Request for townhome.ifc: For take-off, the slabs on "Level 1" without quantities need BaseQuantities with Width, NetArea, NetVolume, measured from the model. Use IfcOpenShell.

First a look at what the model holds.

```python
import ifcopenshell
import ifcopenshell.util.element
import ifcopenshell.util.unit

model = ifcopenshell.open("townhome.ifc")
print(model.schema)
for unit_type in ("LENGTHUNIT", "AREAUNIT", "VOLUMEUNIT"):
    print(unit_type, ifcopenshell.util.unit.calculate_unit_scale(model, unit_type))
storey = next(s for s in model.by_type("IfcBuildingStorey") if s.Name == "Level 1")
slabs = [e for e in ifcopenshell.util.element.get_decomposition(storey) if e.is_a("IfcSlab")]
for e in sorted(slabs, key=lambda e: e.id()):
    print(e.id(), e.is_a(), e.Name, list(ifcopenshell.util.element.get_psets(e, qtos_only=True)), sep=" | ")
```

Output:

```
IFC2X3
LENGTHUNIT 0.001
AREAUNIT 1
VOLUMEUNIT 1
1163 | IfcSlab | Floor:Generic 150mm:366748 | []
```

```python
import ifcopenshell
import ifcopenshell.api.pset
import ifcopenshell.geom
import ifcopenshell.util.element
import ifcopenshell.util.shape
import ifcopenshell.util.unit

model = ifcopenshell.open("townhome.ifc")
unit_scale = ifcopenshell.util.unit.calculate_unit_scale(model)
area_scale = ifcopenshell.util.unit.calculate_unit_scale(model, "AREAUNIT")
volume_scale = ifcopenshell.util.unit.calculate_unit_scale(model, "VOLUMEUNIT")
settings = ifcopenshell.geom.settings()

storey = next(s for s in model.by_type("IfcBuildingStorey") if s.Name == "Level 1")
slabs = [e for e in ifcopenshell.util.element.get_decomposition(storey) if e.is_a("IfcSlab")]

for e in sorted(slabs, key=lambda e: e.id()):
    if ifcopenshell.util.element.get_psets(e, qtos_only=True, should_inherit=False):
        continue
    # Geometry comes back in metres, in the element's own axes.
    shape = ifcopenshell.geom.create_shape(settings, e)
    values = {
        "Width": ifcopenshell.util.shape.get_z(shape.geometry) / unit_scale,
        "NetArea": ifcopenshell.util.shape.get_footprint_area(shape.geometry) / area_scale,
        "NetVolume": ifcopenshell.util.shape.get_volume(shape.geometry) / volume_scale,
    }
    qto = ifcopenshell.api.pset.add_qto(model, product=e, name="BaseQuantities")
    ifcopenshell.api.pset.edit_qto(model, qto=qto, properties=values)
    print(e.id(), {k: round(v, 3) for k, v in values.items()})

model.write("townhome_updated.ifc")
```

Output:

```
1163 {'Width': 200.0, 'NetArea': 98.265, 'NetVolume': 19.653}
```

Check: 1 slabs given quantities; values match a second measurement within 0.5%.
